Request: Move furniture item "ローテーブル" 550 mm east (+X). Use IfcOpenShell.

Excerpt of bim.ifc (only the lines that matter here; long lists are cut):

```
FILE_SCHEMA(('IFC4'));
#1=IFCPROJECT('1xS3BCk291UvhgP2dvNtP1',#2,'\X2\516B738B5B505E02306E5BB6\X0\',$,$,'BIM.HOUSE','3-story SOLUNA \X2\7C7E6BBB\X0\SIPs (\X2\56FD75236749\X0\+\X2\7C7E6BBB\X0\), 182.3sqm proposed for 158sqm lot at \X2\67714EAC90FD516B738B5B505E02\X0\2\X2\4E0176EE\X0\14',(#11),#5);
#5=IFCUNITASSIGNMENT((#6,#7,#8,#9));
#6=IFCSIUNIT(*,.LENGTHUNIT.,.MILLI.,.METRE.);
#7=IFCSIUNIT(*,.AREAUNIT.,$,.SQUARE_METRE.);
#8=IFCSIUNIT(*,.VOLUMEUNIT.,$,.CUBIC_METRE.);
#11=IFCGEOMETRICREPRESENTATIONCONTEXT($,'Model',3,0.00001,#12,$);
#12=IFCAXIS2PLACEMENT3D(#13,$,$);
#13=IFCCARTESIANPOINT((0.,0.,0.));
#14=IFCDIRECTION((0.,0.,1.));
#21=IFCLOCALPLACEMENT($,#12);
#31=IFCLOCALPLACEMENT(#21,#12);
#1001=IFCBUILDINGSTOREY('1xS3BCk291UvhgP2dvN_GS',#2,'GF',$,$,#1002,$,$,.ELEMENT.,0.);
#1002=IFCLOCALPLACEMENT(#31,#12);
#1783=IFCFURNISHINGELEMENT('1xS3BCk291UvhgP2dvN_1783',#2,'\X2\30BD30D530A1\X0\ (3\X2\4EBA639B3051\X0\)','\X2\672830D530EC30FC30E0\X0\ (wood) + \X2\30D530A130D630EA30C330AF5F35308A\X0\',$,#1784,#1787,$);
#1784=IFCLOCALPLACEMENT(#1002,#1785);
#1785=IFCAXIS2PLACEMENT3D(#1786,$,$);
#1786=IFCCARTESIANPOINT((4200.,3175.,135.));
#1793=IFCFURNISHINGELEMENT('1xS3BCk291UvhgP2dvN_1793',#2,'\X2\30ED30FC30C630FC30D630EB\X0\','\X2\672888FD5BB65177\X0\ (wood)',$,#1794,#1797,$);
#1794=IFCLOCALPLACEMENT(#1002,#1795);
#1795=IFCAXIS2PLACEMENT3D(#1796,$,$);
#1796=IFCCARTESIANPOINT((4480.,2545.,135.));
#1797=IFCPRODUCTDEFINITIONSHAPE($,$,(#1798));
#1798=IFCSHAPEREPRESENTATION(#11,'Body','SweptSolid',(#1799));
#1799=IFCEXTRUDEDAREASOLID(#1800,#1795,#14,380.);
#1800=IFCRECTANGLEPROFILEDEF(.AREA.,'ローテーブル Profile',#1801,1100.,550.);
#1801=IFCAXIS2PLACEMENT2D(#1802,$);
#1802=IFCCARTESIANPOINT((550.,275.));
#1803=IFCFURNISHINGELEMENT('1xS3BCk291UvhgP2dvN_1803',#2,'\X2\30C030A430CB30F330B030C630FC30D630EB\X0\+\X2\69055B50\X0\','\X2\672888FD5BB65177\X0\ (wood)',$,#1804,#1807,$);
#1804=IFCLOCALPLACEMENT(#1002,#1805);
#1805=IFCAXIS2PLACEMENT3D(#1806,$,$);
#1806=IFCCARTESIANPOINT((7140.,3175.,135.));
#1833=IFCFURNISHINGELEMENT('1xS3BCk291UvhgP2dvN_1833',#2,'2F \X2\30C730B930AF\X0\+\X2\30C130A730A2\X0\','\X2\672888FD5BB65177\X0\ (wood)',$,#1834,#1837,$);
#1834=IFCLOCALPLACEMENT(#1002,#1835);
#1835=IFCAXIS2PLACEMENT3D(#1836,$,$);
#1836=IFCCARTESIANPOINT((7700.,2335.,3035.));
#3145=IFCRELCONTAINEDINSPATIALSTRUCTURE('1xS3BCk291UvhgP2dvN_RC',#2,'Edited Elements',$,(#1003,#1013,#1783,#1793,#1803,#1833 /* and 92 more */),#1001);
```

```python
import ifcopenshell
import ifcopenshell.api.geometry
import ifcopenshell.util.placement
import ifcopenshell.util.unit

model = ifcopenshell.open("bim.ifc")
unit_scale = ifcopenshell.util.unit.calculate_unit_scale(model)

item = model.by_guid("1xS3BCk291UvhgP2dvN_1793")
matrix = ifcopenshell.util.placement.get_local_placement(item.ObjectPlacement)
matrix[0, 3] += 0.55 / unit_scale
ifcopenshell.api.geometry.edit_object_placement(model, product=item, matrix=matrix, is_si=False)

print(ifcopenshell.util.placement.get_local_placement(item.ObjectPlacement).round(3) + 0.0)

model.write("bim-out.ifc")
```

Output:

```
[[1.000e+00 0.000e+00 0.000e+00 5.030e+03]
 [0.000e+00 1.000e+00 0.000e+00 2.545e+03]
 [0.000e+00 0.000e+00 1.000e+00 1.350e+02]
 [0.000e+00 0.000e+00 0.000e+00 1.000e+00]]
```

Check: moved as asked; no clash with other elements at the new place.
